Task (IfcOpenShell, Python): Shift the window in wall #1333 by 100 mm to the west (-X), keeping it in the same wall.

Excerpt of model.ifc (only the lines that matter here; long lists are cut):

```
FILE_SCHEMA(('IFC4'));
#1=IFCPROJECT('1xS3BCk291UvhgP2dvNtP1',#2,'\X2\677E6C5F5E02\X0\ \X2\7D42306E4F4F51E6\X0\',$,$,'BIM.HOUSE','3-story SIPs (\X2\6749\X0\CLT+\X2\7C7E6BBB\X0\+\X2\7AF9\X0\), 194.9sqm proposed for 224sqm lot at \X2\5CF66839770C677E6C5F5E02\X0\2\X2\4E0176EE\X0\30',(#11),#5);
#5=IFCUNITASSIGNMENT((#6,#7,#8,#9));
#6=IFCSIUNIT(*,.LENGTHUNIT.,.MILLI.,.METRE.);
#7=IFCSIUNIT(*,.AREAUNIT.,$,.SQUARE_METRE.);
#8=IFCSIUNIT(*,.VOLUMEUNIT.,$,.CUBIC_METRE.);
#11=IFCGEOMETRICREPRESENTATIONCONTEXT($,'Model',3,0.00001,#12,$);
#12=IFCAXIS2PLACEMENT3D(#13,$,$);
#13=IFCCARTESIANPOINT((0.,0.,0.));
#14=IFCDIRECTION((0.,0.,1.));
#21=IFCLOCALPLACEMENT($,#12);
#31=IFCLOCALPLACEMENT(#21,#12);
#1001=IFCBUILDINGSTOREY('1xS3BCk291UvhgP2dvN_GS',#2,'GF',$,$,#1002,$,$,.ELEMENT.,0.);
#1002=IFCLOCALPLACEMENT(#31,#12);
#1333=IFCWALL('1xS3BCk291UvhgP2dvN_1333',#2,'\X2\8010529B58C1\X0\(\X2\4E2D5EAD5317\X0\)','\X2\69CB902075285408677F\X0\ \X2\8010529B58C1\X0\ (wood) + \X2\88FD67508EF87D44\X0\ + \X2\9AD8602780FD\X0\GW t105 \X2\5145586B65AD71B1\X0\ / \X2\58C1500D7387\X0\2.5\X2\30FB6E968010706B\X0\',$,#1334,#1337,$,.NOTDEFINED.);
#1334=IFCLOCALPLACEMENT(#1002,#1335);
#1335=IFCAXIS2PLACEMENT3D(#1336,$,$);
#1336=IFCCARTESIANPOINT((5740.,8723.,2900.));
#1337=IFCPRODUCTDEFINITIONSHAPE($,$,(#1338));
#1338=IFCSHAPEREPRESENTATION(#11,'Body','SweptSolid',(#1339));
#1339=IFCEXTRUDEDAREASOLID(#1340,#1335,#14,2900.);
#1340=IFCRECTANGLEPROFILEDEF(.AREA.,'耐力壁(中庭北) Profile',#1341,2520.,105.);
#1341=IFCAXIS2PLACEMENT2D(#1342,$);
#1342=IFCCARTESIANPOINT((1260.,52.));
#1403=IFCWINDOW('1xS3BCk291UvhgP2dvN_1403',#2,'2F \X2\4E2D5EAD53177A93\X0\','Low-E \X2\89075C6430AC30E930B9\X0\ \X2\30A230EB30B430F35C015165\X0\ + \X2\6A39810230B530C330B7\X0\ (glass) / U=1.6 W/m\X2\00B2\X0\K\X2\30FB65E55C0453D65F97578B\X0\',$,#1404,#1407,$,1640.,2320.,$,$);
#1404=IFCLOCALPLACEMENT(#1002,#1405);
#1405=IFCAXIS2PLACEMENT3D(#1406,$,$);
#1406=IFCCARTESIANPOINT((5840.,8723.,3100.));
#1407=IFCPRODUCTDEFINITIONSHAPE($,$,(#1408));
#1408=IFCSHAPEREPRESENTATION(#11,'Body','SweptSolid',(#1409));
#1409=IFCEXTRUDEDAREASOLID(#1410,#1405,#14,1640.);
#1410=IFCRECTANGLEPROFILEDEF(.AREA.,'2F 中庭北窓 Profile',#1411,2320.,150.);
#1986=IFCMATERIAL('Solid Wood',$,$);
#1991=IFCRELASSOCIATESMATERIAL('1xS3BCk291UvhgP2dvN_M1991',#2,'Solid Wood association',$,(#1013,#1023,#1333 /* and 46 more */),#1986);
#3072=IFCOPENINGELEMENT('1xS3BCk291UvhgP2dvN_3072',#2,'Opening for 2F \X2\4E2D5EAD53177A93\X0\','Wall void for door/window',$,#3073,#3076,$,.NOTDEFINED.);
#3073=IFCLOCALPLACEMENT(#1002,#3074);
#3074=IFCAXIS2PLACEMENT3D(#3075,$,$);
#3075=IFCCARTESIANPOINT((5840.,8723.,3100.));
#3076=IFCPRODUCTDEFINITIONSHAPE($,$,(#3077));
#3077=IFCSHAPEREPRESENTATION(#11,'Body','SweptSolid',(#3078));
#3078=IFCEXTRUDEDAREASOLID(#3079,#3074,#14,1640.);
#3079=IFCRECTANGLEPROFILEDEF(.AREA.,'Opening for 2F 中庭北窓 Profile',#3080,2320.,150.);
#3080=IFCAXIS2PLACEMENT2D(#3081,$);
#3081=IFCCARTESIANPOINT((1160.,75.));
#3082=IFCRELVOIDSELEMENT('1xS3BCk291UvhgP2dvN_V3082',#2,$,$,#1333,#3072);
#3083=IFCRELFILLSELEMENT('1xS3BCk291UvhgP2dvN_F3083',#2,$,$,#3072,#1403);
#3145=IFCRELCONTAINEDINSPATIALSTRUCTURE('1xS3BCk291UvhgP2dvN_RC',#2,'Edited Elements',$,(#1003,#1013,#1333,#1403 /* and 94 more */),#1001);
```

```python
import ifcopenshell
import ifcopenshell.api.geometry
import ifcopenshell.util.placement
import ifcopenshell.util.unit

model = ifcopenshell.open("model.ifc")
unit_scale = ifcopenshell.util.unit.calculate_unit_scale(model)

window = model.by_guid("1xS3BCk291UvhgP2dvN_1403")
opening = window.FillsVoids[0].RelatingOpeningElement
wall = opening.VoidsElements[0].RelatingBuildingElement

wall_matrix = ifcopenshell.util.placement.get_local_placement(wall.ObjectPlacement)
shift = wall_matrix[:3, 0] * -0.1 / unit_scale
before = ifcopenshell.util.placement.get_local_placement(window.ObjectPlacement)[:3, 3].copy()

# The window is not placed relative to its opening, so move both.
for product in (opening, window):
    matrix = ifcopenshell.util.placement.get_local_placement(product.ObjectPlacement)
    matrix[:3, 3] += shift
    ifcopenshell.api.geometry.edit_object_placement(model, product=product, matrix=matrix, is_si=False)

after = ifcopenshell.util.placement.get_local_placement(window.ObjectPlacement)[:3, 3]
print("window moved by", (after - before).round(3) + 0.0)

model.write("model_v2.ifc")
```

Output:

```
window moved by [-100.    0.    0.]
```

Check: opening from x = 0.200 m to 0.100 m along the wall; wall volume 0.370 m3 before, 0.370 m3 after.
